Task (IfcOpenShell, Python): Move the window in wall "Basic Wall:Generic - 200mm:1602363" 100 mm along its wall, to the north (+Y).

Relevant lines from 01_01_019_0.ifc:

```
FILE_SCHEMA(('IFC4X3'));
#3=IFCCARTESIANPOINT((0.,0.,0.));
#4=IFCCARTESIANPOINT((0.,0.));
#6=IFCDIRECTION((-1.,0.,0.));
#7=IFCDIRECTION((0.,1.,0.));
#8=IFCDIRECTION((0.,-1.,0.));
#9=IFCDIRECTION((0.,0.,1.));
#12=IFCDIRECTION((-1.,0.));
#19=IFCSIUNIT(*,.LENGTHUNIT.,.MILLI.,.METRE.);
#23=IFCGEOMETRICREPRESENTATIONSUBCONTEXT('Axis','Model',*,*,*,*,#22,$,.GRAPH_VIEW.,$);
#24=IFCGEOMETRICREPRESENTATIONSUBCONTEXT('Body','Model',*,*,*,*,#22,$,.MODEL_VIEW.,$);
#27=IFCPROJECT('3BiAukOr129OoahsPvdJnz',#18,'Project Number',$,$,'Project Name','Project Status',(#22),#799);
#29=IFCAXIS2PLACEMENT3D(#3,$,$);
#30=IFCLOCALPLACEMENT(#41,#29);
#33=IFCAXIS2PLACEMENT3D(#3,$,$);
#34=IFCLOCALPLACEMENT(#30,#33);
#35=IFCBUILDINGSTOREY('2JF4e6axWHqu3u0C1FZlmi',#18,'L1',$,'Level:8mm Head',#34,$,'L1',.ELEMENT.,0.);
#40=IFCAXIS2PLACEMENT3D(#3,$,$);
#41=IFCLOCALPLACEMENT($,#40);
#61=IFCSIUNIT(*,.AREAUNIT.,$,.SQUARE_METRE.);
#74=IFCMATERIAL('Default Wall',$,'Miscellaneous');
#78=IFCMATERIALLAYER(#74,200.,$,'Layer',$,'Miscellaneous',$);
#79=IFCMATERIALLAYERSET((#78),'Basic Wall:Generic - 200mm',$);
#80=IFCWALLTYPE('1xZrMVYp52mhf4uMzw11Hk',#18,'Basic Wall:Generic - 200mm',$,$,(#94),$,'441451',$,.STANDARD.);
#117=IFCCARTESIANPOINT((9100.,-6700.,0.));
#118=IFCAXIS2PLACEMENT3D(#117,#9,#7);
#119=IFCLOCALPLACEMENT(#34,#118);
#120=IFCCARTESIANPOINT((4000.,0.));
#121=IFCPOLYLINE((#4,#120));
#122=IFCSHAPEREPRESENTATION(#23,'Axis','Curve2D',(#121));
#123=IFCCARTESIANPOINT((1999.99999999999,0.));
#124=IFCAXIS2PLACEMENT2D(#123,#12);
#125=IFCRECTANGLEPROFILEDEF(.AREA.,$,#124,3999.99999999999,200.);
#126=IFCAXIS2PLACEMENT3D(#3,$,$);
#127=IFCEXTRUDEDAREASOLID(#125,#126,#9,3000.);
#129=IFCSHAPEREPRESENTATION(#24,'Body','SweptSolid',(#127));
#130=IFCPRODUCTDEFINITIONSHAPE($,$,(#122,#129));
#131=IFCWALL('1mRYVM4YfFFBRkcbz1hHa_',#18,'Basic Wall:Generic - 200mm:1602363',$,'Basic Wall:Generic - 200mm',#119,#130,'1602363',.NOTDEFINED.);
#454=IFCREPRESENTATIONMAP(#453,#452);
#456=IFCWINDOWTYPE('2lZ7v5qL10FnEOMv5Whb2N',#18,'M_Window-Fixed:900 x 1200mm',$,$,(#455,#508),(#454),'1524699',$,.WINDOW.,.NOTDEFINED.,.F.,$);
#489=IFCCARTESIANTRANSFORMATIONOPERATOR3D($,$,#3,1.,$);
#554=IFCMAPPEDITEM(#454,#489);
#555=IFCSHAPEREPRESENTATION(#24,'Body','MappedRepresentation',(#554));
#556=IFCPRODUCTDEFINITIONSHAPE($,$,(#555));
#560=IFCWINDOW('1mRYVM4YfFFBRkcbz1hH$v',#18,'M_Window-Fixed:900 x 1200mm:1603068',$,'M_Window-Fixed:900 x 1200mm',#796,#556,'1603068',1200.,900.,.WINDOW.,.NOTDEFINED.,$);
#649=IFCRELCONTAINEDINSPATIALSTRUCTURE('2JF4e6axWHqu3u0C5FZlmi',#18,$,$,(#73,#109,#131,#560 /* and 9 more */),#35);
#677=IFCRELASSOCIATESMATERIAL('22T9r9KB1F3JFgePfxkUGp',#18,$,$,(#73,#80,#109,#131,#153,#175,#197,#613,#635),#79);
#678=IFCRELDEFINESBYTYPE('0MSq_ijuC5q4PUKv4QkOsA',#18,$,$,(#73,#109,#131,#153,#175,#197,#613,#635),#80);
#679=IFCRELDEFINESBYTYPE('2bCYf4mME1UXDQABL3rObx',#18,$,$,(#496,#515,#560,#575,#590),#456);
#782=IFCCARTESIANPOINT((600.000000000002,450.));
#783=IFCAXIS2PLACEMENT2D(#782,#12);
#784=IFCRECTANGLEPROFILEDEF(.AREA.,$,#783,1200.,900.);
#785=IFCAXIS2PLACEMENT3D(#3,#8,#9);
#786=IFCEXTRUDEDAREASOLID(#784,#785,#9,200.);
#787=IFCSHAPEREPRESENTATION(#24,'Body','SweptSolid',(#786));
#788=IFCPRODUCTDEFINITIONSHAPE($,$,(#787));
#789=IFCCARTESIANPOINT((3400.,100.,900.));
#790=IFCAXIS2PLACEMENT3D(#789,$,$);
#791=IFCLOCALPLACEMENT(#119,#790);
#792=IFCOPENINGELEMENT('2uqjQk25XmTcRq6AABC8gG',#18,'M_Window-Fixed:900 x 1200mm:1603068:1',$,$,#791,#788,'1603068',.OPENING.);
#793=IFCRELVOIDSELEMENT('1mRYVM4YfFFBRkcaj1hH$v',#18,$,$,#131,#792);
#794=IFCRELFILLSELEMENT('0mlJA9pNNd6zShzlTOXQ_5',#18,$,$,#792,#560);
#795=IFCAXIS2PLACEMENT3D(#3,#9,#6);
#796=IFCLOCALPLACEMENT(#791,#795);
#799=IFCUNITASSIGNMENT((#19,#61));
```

```python
import ifcopenshell
import ifcopenshell.api.geometry
import ifcopenshell.util.placement
import ifcopenshell.util.unit

model = ifcopenshell.open("01_01_019_0.ifc")
unit_scale = ifcopenshell.util.unit.calculate_unit_scale(model)

window = model.by_guid("1mRYVM4YfFFBRkcbz1hH$v")
opening = window.FillsVoids[0].RelatingOpeningElement
wall = opening.VoidsElements[0].RelatingBuildingElement

wall_matrix = ifcopenshell.util.placement.get_local_placement(wall.ObjectPlacement)
shift = wall_matrix[:3, 0] * 0.1 / unit_scale
before = ifcopenshell.util.placement.get_local_placement(window.ObjectPlacement)[:3, 3].copy()

# The window is placed relative to its opening, so it follows when the opening moves.
matrix = ifcopenshell.util.placement.get_local_placement(opening.ObjectPlacement)
matrix[:3, 3] += shift
ifcopenshell.api.geometry.edit_object_placement(
    model, product=opening, matrix=matrix, is_si=False, should_transform_children=True
)

after = ifcopenshell.util.placement.get_local_placement(window.ObjectPlacement)[:3, 3]
print("window moved by", (after - before).round(3) + 0.0)

model.write("01_01_019_0_edited.ifc")
```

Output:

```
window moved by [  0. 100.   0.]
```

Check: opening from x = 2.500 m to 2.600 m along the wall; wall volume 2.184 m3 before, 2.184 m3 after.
